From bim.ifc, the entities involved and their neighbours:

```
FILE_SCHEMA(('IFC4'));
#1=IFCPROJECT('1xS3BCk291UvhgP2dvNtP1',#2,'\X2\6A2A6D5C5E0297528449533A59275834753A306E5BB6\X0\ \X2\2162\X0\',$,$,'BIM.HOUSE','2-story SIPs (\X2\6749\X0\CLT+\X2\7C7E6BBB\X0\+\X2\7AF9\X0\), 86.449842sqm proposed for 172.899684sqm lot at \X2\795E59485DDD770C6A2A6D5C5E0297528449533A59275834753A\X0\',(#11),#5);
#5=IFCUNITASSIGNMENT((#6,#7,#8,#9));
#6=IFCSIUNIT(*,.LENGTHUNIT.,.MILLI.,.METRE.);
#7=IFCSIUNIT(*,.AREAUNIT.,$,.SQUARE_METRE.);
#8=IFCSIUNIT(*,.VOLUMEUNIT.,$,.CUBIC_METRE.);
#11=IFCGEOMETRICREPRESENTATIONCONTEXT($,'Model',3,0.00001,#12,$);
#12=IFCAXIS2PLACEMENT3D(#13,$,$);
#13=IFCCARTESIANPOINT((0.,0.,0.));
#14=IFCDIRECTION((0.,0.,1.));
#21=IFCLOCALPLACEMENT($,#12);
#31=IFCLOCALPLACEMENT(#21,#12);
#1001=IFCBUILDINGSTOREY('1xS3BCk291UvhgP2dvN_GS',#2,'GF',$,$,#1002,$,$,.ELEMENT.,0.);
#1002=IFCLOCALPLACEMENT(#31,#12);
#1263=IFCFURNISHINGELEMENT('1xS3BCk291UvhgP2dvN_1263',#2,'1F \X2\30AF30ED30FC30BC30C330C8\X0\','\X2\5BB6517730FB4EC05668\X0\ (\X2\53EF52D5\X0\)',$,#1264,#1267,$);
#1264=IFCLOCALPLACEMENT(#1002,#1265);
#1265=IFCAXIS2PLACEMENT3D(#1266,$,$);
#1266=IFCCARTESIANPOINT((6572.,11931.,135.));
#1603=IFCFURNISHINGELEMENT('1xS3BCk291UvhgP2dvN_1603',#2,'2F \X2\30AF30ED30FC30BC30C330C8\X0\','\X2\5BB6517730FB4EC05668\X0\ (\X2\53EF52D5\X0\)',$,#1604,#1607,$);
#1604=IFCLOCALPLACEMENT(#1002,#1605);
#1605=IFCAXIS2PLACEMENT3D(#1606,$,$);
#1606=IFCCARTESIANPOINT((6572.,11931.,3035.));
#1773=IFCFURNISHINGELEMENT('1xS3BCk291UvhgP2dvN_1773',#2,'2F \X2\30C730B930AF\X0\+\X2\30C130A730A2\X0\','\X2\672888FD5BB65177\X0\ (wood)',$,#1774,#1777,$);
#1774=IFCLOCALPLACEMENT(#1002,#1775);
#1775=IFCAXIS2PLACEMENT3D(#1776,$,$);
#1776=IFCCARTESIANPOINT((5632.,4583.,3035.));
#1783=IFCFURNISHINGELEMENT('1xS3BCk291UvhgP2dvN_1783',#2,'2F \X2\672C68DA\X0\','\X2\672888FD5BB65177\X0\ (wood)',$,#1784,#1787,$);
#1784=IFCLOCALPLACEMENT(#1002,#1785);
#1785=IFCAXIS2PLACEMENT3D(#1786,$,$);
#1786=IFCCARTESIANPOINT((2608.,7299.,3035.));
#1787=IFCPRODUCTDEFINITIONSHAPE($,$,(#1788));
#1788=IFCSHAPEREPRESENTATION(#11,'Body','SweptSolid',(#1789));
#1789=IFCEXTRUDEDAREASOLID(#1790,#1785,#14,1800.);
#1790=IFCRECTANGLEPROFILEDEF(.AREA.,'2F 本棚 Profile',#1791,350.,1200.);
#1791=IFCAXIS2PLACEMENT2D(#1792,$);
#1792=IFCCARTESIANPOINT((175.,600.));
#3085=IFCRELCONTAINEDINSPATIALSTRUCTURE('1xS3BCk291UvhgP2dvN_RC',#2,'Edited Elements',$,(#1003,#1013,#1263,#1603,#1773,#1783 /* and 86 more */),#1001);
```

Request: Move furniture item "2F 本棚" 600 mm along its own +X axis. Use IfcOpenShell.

```python
import ifcopenshell
import ifcopenshell.api.geometry
import ifcopenshell.util.placement
import ifcopenshell.util.unit

model = ifcopenshell.open("bim.ifc")
unit_scale = ifcopenshell.util.unit.calculate_unit_scale(model)

item = model.by_guid("1xS3BCk291UvhgP2dvN_1783")
matrix = ifcopenshell.util.placement.get_local_placement(item.ObjectPlacement)
matrix[:3, 3] += matrix[:3, 0] * 0.6 / unit_scale
ifcopenshell.api.geometry.edit_object_placement(model, product=item, matrix=matrix, is_si=False)

print(ifcopenshell.util.placement.get_local_placement(item.ObjectPlacement).round(3) + 0.0)

model.write("bim_v2.ifc")
```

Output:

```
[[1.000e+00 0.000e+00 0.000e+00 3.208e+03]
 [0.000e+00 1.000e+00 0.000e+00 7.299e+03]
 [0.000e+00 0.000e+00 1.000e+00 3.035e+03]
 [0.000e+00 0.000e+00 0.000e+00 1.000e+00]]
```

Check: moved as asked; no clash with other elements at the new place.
